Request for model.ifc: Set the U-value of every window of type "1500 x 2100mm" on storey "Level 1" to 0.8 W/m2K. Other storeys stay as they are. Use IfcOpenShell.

First a look at what the model holds.

```python
import ifcopenshell
import ifcopenshell.util.element

model = ifcopenshell.open("model.ifc")
print(model.schema)
storey = next(s for s in model.by_type("IfcBuildingStorey") if s.Name == "Level 1")
windows = [e for e in ifcopenshell.util.element.get_decomposition(storey) if e.is_a("IfcWindow")]
seen = {}
for e in windows:
    element_type = ifcopenshell.util.element.get_type(e)
    key = (element_type.Name if element_type != e and element_type else None, ifcopenshell.util.element.get_pset(e, "Pset_WindowCommon", "ThermalTransmittance"))
    seen[key] = seen.get(key, 0) + 1
for (name, value), count in sorted(seen.items(), key=str):
    print(count, "x", name, "|", value)
```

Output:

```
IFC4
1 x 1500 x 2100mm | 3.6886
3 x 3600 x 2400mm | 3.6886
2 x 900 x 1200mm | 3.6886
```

```python
import ifcopenshell
import ifcopenshell.api.pset
import ifcopenshell.util.element

model = ifcopenshell.open("model.ifc")

storey = next(s for s in model.by_type("IfcBuildingStorey") if s.Name == "Level 1")
windows = [e for e in ifcopenshell.util.element.get_decomposition(storey) if e.is_a("IfcWindow")]

count = 0
for e in windows:
    element_type = ifcopenshell.util.element.get_type(e)
    if element_type in (None, e) or element_type.Name != "1500 x 2100mm":
        continue
    # add_pset returns the element's existing set when there is one.
    pset = ifcopenshell.api.pset.add_pset(model, product=e, name="Pset_WindowCommon")
    ifcopenshell.api.pset.edit_pset(model, pset=pset, properties={"ThermalTransmittance": 0.8})
    count += 1

print(count, "windows updated")

model.write("model-out.ifc")
```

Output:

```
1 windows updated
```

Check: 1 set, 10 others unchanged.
